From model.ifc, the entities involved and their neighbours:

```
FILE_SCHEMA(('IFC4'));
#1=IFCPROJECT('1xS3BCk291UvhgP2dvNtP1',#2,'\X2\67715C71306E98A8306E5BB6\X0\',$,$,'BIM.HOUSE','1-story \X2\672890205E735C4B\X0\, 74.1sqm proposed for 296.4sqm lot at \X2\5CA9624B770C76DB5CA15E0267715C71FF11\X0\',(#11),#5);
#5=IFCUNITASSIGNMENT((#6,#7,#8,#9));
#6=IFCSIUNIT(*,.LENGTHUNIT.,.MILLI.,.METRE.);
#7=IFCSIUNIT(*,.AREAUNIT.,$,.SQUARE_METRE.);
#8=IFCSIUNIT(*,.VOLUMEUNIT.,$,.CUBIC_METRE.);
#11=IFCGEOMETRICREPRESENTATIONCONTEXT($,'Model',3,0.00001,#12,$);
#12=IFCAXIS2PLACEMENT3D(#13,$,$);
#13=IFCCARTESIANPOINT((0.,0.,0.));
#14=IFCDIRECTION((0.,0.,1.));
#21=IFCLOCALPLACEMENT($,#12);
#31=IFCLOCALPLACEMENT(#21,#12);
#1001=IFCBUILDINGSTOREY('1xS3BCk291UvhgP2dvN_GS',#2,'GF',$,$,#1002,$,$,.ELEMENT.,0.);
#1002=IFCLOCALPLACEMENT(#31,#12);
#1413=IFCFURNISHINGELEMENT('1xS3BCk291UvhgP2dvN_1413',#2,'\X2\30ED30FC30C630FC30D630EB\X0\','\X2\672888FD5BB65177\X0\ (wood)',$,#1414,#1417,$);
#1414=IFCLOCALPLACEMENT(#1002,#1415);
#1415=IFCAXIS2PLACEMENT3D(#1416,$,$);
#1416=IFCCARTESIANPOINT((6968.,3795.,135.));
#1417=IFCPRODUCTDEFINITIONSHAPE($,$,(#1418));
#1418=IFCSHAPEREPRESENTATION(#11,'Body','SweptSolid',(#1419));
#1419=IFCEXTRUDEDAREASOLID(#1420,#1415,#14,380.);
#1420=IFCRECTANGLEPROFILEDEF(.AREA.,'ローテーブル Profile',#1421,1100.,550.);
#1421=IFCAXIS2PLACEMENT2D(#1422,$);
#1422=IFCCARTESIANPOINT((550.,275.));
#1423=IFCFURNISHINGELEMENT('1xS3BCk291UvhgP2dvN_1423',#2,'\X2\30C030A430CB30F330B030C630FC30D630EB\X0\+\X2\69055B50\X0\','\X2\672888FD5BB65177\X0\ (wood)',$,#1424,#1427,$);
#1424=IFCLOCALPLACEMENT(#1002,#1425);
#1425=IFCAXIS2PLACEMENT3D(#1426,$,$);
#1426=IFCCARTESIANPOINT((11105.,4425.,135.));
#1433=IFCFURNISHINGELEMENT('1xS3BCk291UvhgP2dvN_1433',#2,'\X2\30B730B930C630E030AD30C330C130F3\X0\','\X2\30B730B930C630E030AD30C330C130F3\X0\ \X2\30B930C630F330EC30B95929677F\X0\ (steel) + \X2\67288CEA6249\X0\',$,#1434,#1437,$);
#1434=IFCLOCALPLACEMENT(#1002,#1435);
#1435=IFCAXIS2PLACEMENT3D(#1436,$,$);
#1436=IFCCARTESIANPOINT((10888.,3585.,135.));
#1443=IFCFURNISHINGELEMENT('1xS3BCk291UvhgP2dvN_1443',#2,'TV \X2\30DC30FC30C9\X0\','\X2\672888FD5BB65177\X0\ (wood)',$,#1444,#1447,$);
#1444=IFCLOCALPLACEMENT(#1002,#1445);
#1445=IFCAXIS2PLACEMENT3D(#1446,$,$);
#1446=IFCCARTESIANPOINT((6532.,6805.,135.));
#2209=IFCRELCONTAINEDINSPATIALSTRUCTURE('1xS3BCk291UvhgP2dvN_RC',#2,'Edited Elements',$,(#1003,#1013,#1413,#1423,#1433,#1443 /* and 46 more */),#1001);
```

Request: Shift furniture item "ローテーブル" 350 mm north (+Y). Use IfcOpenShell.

```python
import ifcopenshell
import ifcopenshell.api.geometry
import ifcopenshell.util.placement
import ifcopenshell.util.unit

model = ifcopenshell.open("model.ifc")
unit_scale = ifcopenshell.util.unit.calculate_unit_scale(model)

item = model.by_guid("1xS3BCk291UvhgP2dvN_1413")
matrix = ifcopenshell.util.placement.get_local_placement(item.ObjectPlacement)
matrix[1, 3] += 0.35 / unit_scale
ifcopenshell.api.geometry.edit_object_placement(model, product=item, matrix=matrix, is_si=False)

print(ifcopenshell.util.placement.get_local_placement(item.ObjectPlacement).round(3) + 0.0)

model.write("model_rev.ifc")
```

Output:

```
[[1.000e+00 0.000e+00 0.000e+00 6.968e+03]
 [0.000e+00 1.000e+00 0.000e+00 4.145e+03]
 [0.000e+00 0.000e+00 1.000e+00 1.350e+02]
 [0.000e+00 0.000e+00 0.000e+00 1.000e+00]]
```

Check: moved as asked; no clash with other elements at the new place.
